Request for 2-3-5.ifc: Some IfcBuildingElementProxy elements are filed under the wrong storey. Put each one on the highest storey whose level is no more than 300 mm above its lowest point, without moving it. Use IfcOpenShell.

First a look at what the model holds.

```python
import ifcopenshell
import ifcopenshell.util.element
import ifcopenshell.util.placement

model = ifcopenshell.open("2-3-5.ifc")
print(model.schema)
for storey in model.by_type("IfcBuildingStorey"):
    level = ifcopenshell.util.placement.get_storey_elevation(storey)
    count = sum(e.is_a("IfcBuildingElementProxy") for e in ifcopenshell.util.element.get_contained(storey))
    print(storey.id(), storey.Name, round(level, 3), count, sep=" | ")
```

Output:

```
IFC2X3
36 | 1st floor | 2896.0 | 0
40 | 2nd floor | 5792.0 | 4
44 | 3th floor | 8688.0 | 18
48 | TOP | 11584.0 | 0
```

```python
import ifcopenshell
import ifcopenshell.api.spatial
import ifcopenshell.geom
import ifcopenshell.util.element
import ifcopenshell.util.placement
import ifcopenshell.util.shape
import ifcopenshell.util.unit

model = ifcopenshell.open("2-3-5.ifc")
unit_scale = ifcopenshell.util.unit.calculate_unit_scale(model)
settings = ifcopenshell.geom.settings()

levels = sorted(
    ((ifcopenshell.util.placement.get_storey_elevation(s) * unit_scale, s) for s in model.by_type("IfcBuildingStorey")),
    key=lambda pair: pair[0],
)

for e in model.by_type("IfcBuildingElementProxy"):
    current = e.ContainedInStructure[0].RelatingStructure if e.ContainedInStructure else None
    if current is None or not current.is_a("IfcBuildingStorey"):
        continue
    shape = ifcopenshell.geom.create_shape(settings, e)
    bottom = ifcopenshell.util.shape.get_shape_bottom_elevation(shape, shape.geometry)
    below = [s for level, s in levels if level <= bottom + 0.3]
    storey = below[-1] if below else levels[0][1]
    if storey != current:
        # assign_container keeps the world position.
        ifcopenshell.api.spatial.assign_container(model, products=[e], relating_structure=storey)
        print(e.id(), current.Name, "->", storey.Name)

model.write("2-3-5_updated.ifc")
```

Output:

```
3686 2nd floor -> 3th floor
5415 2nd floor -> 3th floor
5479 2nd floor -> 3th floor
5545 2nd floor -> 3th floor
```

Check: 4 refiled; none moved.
